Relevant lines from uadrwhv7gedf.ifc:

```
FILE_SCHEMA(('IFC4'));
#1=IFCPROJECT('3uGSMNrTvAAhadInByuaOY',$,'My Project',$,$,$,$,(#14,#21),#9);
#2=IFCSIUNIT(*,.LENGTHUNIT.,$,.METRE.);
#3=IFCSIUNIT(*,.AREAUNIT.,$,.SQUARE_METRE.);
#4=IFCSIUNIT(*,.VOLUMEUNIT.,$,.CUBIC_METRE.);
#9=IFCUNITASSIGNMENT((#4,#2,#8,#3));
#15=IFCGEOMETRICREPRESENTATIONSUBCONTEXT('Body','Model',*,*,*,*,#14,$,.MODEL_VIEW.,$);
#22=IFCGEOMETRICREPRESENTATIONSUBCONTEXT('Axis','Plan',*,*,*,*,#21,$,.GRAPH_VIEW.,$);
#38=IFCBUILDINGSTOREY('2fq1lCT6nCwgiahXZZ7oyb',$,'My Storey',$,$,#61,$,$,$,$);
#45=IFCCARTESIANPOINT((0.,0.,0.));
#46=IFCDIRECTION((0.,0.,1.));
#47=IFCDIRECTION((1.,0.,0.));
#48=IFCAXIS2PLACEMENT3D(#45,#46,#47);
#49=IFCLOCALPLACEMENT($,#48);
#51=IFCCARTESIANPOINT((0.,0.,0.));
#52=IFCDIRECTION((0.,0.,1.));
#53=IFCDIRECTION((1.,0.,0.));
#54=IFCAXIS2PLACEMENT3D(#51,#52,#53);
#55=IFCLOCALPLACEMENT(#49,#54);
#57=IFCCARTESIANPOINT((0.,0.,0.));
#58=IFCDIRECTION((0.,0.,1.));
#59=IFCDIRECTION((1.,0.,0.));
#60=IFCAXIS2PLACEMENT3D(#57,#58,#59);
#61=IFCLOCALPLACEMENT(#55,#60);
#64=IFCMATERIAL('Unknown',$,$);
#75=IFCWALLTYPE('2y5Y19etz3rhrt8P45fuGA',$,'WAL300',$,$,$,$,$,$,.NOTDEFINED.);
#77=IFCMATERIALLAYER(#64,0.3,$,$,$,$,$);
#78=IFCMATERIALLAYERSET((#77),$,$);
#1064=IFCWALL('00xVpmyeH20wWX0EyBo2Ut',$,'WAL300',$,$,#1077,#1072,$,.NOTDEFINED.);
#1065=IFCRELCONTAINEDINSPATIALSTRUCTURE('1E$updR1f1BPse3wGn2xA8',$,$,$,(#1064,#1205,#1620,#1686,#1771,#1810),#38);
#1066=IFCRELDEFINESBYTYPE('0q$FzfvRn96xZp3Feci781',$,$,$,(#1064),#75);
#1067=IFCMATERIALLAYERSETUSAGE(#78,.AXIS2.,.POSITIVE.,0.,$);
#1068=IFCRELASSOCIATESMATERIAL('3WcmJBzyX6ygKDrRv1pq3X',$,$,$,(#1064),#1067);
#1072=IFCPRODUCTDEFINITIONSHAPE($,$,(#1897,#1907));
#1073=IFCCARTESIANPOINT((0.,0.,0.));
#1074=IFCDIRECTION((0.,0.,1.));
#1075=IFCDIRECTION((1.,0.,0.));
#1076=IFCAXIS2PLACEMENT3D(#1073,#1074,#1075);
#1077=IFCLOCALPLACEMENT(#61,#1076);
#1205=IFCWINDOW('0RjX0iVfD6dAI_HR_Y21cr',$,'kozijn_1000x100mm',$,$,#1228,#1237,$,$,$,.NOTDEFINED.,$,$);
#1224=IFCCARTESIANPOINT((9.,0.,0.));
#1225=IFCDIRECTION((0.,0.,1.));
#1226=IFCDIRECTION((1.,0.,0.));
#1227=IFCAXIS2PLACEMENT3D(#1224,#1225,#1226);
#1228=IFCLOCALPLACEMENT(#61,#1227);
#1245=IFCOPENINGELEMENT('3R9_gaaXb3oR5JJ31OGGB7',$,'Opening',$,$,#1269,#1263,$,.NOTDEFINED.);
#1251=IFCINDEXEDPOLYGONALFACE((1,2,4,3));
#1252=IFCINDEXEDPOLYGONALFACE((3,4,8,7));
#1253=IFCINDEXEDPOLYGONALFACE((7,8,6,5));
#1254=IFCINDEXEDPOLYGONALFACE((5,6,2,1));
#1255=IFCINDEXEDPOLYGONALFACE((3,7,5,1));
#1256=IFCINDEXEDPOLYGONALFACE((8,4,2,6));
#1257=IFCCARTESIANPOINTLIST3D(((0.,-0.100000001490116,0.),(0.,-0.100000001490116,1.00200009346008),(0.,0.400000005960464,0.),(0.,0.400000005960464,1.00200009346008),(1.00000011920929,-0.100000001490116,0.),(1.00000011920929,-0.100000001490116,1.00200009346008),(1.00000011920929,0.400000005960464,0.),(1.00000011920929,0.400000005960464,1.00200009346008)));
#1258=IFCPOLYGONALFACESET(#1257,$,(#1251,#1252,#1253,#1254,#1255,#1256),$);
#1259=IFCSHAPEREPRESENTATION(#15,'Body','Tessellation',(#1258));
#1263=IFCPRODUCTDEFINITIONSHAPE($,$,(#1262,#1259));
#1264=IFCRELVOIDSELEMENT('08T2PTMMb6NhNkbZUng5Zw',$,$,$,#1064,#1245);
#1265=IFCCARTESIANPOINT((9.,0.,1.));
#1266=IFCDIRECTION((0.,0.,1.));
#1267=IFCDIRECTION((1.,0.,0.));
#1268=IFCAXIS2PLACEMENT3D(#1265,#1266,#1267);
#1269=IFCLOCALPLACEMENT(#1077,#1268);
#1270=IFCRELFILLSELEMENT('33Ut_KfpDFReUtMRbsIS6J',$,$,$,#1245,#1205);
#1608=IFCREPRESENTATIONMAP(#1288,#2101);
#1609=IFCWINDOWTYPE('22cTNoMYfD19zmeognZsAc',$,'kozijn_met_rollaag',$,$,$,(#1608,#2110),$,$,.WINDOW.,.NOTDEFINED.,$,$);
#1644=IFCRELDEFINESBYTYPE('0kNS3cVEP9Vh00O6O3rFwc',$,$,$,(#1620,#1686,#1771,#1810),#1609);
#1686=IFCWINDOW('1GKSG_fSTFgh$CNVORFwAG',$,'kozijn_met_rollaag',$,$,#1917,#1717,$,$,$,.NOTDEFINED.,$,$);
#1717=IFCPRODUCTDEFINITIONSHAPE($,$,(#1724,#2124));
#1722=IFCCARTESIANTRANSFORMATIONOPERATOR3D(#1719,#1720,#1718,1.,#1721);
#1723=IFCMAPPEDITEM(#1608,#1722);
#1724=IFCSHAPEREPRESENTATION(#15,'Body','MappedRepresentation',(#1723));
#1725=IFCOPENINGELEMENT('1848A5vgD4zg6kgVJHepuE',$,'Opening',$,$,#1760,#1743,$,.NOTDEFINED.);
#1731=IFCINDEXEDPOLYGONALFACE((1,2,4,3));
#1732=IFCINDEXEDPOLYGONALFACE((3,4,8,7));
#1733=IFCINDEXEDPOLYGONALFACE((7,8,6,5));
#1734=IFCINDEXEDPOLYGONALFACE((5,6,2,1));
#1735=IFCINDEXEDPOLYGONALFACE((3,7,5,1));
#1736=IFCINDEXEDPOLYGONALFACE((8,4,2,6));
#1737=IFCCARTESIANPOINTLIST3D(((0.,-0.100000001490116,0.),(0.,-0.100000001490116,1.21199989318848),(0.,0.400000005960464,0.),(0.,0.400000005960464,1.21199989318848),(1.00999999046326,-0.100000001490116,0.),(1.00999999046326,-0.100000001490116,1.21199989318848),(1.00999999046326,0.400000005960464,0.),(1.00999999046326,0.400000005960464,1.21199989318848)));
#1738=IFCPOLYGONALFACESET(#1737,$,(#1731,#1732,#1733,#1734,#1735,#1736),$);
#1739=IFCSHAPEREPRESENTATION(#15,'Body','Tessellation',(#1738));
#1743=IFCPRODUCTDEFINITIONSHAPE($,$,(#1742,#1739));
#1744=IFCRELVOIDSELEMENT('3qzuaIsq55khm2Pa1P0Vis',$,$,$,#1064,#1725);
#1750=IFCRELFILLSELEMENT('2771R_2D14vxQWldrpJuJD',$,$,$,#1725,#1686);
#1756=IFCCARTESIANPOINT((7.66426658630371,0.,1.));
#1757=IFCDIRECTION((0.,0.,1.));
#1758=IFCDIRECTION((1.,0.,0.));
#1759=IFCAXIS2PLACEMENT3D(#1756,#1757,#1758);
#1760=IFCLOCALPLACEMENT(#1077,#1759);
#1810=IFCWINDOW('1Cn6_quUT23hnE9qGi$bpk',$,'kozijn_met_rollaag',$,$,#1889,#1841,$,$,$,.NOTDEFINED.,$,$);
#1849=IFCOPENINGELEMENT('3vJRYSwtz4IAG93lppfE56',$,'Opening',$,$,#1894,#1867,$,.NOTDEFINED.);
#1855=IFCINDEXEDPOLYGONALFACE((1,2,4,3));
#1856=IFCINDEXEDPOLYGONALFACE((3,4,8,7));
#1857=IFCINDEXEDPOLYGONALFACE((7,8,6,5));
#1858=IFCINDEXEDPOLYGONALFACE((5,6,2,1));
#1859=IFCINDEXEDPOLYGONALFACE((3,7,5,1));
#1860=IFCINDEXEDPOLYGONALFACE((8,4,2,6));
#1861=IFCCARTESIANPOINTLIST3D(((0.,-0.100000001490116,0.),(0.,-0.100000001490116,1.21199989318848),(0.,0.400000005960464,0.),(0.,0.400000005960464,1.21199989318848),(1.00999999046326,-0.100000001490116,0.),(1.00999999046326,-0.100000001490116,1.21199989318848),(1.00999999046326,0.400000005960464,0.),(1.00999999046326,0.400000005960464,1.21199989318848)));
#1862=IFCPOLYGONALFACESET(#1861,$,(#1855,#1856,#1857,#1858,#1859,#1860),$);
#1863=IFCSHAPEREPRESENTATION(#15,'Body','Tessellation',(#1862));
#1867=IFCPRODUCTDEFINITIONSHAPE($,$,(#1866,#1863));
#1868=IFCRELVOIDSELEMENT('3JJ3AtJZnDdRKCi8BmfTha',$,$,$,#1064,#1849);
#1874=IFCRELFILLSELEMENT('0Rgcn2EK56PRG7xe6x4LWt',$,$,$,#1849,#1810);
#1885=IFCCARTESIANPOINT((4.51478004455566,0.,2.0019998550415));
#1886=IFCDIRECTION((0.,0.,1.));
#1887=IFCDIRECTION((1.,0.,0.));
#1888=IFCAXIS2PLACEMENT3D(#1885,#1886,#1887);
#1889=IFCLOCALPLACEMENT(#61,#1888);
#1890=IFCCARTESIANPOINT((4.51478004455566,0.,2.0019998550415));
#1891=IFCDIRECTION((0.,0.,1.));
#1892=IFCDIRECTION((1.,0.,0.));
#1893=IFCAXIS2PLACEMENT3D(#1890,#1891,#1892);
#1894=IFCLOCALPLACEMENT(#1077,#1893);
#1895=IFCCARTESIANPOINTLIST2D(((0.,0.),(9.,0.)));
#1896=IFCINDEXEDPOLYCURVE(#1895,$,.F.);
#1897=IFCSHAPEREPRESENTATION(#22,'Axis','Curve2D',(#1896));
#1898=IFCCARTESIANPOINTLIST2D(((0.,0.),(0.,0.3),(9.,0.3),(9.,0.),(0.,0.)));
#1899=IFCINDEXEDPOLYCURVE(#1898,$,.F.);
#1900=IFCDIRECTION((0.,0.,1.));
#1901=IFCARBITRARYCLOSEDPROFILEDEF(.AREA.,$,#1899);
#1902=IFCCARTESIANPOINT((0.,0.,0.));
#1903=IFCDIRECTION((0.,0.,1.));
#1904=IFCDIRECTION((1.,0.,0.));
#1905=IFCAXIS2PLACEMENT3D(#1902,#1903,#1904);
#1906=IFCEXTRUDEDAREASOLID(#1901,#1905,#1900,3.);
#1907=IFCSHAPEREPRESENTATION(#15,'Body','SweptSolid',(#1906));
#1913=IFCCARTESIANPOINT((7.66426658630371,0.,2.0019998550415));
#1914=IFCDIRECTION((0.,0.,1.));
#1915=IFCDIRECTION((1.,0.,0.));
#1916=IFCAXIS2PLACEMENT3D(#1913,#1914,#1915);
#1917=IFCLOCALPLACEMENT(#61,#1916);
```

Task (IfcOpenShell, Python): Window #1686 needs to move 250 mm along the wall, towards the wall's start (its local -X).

```python
import ifcopenshell
import ifcopenshell.api.geometry
import ifcopenshell.util.placement

model = ifcopenshell.open("uadrwhv7gedf.ifc")

window = model.by_guid("1GKSG_fSTFgh$CNVORFwAG")
opening = window.FillsVoids[0].RelatingOpeningElement
wall = opening.VoidsElements[0].RelatingBuildingElement

wall_matrix = ifcopenshell.util.placement.get_local_placement(wall.ObjectPlacement)
shift = wall_matrix[:3, 0] * -0.25
before = ifcopenshell.util.placement.get_local_placement(window.ObjectPlacement)[:3, 3].copy()

# The window is not placed relative to its opening, so move both.
for product in (opening, window):
    matrix = ifcopenshell.util.placement.get_local_placement(product.ObjectPlacement)
    matrix[:3, 3] += shift
    ifcopenshell.api.geometry.edit_object_placement(model, product=product, matrix=matrix, is_si=False)

after = ifcopenshell.util.placement.get_local_placement(window.ObjectPlacement)[:3, 3]
print("window moved by", (after - before).round(3) + 0.0)

model.write("uadrwhv7gedf_edited.ifc")
```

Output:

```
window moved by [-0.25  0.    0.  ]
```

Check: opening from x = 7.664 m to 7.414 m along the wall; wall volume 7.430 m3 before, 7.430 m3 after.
